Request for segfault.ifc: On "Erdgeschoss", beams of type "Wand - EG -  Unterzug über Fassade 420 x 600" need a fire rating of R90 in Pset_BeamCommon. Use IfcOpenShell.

First a look at what the model holds.

```python
import ifcopenshell
import ifcopenshell.util.element

model = ifcopenshell.open("segfault.ifc")
print(model.schema)
storey = next(s for s in model.by_type("IfcBuildingStorey") if s.Name == "Erdgeschoss")
beams = [e for e in ifcopenshell.util.element.get_decomposition(storey) if e.is_a("IfcBeam")]
seen = {}
for e in beams:
    element_type = ifcopenshell.util.element.get_type(e)
    key = (element_type.Name if element_type != e and element_type else None, ifcopenshell.util.element.get_pset(e, "Pset_BeamCommon", "FireRating"))
    seen[key] = seen.get(key, 0) + 1
for (name, value), count in sorted(seen.items(), key=str):
    print(count, "x", name, "|", value)
```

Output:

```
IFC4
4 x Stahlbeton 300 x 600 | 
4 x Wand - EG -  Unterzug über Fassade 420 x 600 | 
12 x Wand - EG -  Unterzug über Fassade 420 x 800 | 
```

```python
import ifcopenshell
import ifcopenshell.api.pset
import ifcopenshell.util.element

model = ifcopenshell.open("segfault.ifc")

storey = next(s for s in model.by_type("IfcBuildingStorey") if s.Name == "Erdgeschoss")
beams = [e for e in ifcopenshell.util.element.get_decomposition(storey) if e.is_a("IfcBeam")]

count = 0
for e in beams:
    element_type = ifcopenshell.util.element.get_type(e)
    if element_type in (None, e) or element_type.Name != "Wand - EG -  Unterzug über Fassade 420 x 600":
        continue
    # add_pset returns the element's existing set when there is one.
    pset = ifcopenshell.api.pset.add_pset(model, product=e, name="Pset_BeamCommon")
    ifcopenshell.api.pset.edit_pset(model, pset=pset, properties={"FireRating": "R90"})
    count += 1

print(count, "beams updated")

model.write("segfault_updated.ifc")
```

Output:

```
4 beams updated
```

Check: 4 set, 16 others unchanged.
